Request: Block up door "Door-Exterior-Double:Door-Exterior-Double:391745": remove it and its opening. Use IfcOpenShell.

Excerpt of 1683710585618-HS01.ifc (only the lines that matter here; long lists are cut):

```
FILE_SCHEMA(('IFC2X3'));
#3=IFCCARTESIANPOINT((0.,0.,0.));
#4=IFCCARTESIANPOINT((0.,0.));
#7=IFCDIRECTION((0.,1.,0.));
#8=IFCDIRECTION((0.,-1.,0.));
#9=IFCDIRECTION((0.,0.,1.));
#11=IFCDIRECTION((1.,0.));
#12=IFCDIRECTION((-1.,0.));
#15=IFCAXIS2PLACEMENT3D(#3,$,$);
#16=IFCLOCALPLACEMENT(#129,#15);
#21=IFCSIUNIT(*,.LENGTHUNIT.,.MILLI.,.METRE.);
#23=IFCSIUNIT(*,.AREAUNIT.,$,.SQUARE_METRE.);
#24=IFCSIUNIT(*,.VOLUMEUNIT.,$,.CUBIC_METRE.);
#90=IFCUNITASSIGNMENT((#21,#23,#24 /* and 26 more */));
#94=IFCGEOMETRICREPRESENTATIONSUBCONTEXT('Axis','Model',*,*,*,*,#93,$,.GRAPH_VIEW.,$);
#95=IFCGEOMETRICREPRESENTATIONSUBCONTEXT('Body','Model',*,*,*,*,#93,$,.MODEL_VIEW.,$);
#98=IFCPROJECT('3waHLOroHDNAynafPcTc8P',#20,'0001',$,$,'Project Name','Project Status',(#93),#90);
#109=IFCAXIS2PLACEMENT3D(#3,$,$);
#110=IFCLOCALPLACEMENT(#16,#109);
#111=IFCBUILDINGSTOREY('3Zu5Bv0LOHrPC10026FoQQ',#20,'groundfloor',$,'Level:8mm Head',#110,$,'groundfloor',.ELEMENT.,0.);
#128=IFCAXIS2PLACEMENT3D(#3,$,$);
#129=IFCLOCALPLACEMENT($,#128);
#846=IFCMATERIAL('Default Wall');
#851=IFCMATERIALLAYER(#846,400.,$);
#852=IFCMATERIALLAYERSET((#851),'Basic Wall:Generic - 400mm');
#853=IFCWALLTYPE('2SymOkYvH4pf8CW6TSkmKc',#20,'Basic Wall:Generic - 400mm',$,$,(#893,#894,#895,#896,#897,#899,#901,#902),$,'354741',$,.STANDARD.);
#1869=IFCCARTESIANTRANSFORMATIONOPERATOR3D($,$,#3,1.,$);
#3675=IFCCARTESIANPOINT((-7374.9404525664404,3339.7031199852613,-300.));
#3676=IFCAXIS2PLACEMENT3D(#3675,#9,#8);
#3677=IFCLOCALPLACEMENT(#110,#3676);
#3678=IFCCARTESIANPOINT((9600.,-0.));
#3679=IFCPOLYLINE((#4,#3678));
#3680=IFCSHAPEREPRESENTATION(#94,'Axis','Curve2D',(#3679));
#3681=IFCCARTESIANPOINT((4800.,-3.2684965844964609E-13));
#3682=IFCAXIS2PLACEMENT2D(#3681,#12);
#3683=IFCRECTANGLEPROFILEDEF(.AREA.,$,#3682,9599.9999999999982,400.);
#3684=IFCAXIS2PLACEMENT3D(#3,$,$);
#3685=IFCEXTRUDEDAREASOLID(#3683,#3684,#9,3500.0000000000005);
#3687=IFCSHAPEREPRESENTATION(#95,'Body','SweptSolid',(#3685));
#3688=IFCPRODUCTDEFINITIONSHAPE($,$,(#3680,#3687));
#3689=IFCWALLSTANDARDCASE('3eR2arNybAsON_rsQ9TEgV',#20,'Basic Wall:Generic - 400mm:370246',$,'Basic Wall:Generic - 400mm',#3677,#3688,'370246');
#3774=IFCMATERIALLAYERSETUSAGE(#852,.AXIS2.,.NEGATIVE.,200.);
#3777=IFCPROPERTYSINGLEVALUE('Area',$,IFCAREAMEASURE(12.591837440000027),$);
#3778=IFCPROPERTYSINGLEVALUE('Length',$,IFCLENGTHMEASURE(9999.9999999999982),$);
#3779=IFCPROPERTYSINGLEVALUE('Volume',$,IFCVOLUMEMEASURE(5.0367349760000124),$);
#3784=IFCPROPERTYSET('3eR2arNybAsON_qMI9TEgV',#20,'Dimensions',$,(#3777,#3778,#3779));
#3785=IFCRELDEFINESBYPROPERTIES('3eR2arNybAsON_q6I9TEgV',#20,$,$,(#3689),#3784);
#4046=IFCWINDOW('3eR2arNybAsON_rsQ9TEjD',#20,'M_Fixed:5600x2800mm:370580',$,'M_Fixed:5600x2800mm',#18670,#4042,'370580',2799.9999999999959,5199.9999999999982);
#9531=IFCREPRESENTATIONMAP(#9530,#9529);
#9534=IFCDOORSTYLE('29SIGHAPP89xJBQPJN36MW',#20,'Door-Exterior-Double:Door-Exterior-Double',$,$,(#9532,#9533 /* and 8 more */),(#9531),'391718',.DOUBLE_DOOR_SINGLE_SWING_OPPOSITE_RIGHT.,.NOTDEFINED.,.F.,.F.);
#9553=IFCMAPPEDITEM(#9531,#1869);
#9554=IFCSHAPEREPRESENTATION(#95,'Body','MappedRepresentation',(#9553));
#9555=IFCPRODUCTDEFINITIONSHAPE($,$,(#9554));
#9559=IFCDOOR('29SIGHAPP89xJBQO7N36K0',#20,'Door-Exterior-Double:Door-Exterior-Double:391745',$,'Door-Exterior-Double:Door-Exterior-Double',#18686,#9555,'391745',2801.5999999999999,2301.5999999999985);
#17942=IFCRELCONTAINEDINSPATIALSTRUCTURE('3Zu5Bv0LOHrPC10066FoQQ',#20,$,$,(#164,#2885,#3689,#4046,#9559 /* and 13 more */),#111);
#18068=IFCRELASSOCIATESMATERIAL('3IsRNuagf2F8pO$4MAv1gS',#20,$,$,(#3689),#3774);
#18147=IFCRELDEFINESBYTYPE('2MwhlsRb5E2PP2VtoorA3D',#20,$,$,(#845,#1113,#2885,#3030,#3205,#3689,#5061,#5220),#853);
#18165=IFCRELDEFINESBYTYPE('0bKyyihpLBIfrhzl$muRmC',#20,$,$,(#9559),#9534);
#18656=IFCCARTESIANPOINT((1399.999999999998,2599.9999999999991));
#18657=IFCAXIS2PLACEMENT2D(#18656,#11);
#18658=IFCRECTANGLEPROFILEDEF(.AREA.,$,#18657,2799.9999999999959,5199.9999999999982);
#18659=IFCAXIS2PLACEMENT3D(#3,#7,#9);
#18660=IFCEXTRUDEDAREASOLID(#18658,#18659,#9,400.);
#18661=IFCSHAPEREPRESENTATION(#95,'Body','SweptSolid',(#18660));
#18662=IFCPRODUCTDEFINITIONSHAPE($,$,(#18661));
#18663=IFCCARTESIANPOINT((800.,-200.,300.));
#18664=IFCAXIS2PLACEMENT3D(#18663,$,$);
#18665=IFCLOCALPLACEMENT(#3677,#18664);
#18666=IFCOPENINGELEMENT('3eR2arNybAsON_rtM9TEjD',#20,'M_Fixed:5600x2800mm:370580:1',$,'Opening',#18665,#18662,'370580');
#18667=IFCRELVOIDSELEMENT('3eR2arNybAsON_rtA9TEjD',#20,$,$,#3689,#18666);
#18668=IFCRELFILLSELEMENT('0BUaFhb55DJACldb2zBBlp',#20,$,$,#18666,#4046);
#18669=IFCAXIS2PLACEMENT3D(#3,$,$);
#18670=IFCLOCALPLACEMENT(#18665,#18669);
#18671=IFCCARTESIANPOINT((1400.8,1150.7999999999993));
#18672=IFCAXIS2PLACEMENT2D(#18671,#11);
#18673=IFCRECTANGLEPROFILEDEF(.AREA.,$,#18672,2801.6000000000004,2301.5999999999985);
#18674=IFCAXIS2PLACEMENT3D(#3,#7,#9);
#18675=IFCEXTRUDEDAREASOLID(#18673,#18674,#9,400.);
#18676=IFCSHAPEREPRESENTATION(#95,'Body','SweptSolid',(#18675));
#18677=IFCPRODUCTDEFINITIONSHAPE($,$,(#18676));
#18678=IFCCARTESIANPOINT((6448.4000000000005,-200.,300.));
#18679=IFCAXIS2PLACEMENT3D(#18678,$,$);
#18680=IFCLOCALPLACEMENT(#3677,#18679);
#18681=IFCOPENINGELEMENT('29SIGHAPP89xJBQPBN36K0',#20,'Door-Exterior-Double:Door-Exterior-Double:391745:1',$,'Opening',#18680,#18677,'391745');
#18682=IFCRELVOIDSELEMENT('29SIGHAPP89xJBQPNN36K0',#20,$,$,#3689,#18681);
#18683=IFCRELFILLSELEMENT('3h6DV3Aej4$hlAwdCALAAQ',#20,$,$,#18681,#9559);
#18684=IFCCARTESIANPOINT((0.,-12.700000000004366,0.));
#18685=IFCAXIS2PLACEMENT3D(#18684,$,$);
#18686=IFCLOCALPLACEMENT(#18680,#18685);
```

```python
import ifcopenshell
import ifcopenshell.api.feature
import ifcopenshell.api.pset
import ifcopenshell.api.root
import ifcopenshell.geom
import ifcopenshell.util.element
import ifcopenshell.util.shape
import ifcopenshell.util.unit

model = ifcopenshell.open("1683710585618-HS01.ifc")
area_scale = ifcopenshell.util.unit.calculate_unit_scale(model, "AREAUNIT")
volume_scale = ifcopenshell.util.unit.calculate_unit_scale(model, "VOLUMEUNIT")
settings = ifcopenshell.geom.settings()


def volume(element):
    """Net volume in cubic metres, openings subtracted."""
    shape = ifcopenshell.geom.create_shape(settings, element)
    return ifcopenshell.util.shape.get_volume(shape.geometry)


door = model.by_guid("29SIGHAPP89xJBQO7N36K0")
opening = door.FillsVoids[0].RelatingOpeningElement
wall = opening.VoidsElements[0].RelatingBuildingElement
before = volume(wall)

ifcopenshell.api.root.remove_product(model, product=door)
ifcopenshell.api.feature.remove_feature(model, feature=opening)

after = volume(wall)
thickness = 0.4  # wall thickness in metres

# Update the wall's stored quantities.
pset = model.by_id(ifcopenshell.util.element.get_pset(wall, "Dimensions", should_inherit=False)["id"])
ifcopenshell.api.pset.edit_pset(model, pset=pset, properties={
    "Area": model.create_entity("IfcAreaMeasure", after / thickness / area_scale),
    "Volume": model.create_entity("IfcVolumeMeasure", after / volume_scale),
})

print(f"wall volume {before:.3f} -> {after:.3f} m3")

model.write("1683710585618-HS01_rev.ifc")
```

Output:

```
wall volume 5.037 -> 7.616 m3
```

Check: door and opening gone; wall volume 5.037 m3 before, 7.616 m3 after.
